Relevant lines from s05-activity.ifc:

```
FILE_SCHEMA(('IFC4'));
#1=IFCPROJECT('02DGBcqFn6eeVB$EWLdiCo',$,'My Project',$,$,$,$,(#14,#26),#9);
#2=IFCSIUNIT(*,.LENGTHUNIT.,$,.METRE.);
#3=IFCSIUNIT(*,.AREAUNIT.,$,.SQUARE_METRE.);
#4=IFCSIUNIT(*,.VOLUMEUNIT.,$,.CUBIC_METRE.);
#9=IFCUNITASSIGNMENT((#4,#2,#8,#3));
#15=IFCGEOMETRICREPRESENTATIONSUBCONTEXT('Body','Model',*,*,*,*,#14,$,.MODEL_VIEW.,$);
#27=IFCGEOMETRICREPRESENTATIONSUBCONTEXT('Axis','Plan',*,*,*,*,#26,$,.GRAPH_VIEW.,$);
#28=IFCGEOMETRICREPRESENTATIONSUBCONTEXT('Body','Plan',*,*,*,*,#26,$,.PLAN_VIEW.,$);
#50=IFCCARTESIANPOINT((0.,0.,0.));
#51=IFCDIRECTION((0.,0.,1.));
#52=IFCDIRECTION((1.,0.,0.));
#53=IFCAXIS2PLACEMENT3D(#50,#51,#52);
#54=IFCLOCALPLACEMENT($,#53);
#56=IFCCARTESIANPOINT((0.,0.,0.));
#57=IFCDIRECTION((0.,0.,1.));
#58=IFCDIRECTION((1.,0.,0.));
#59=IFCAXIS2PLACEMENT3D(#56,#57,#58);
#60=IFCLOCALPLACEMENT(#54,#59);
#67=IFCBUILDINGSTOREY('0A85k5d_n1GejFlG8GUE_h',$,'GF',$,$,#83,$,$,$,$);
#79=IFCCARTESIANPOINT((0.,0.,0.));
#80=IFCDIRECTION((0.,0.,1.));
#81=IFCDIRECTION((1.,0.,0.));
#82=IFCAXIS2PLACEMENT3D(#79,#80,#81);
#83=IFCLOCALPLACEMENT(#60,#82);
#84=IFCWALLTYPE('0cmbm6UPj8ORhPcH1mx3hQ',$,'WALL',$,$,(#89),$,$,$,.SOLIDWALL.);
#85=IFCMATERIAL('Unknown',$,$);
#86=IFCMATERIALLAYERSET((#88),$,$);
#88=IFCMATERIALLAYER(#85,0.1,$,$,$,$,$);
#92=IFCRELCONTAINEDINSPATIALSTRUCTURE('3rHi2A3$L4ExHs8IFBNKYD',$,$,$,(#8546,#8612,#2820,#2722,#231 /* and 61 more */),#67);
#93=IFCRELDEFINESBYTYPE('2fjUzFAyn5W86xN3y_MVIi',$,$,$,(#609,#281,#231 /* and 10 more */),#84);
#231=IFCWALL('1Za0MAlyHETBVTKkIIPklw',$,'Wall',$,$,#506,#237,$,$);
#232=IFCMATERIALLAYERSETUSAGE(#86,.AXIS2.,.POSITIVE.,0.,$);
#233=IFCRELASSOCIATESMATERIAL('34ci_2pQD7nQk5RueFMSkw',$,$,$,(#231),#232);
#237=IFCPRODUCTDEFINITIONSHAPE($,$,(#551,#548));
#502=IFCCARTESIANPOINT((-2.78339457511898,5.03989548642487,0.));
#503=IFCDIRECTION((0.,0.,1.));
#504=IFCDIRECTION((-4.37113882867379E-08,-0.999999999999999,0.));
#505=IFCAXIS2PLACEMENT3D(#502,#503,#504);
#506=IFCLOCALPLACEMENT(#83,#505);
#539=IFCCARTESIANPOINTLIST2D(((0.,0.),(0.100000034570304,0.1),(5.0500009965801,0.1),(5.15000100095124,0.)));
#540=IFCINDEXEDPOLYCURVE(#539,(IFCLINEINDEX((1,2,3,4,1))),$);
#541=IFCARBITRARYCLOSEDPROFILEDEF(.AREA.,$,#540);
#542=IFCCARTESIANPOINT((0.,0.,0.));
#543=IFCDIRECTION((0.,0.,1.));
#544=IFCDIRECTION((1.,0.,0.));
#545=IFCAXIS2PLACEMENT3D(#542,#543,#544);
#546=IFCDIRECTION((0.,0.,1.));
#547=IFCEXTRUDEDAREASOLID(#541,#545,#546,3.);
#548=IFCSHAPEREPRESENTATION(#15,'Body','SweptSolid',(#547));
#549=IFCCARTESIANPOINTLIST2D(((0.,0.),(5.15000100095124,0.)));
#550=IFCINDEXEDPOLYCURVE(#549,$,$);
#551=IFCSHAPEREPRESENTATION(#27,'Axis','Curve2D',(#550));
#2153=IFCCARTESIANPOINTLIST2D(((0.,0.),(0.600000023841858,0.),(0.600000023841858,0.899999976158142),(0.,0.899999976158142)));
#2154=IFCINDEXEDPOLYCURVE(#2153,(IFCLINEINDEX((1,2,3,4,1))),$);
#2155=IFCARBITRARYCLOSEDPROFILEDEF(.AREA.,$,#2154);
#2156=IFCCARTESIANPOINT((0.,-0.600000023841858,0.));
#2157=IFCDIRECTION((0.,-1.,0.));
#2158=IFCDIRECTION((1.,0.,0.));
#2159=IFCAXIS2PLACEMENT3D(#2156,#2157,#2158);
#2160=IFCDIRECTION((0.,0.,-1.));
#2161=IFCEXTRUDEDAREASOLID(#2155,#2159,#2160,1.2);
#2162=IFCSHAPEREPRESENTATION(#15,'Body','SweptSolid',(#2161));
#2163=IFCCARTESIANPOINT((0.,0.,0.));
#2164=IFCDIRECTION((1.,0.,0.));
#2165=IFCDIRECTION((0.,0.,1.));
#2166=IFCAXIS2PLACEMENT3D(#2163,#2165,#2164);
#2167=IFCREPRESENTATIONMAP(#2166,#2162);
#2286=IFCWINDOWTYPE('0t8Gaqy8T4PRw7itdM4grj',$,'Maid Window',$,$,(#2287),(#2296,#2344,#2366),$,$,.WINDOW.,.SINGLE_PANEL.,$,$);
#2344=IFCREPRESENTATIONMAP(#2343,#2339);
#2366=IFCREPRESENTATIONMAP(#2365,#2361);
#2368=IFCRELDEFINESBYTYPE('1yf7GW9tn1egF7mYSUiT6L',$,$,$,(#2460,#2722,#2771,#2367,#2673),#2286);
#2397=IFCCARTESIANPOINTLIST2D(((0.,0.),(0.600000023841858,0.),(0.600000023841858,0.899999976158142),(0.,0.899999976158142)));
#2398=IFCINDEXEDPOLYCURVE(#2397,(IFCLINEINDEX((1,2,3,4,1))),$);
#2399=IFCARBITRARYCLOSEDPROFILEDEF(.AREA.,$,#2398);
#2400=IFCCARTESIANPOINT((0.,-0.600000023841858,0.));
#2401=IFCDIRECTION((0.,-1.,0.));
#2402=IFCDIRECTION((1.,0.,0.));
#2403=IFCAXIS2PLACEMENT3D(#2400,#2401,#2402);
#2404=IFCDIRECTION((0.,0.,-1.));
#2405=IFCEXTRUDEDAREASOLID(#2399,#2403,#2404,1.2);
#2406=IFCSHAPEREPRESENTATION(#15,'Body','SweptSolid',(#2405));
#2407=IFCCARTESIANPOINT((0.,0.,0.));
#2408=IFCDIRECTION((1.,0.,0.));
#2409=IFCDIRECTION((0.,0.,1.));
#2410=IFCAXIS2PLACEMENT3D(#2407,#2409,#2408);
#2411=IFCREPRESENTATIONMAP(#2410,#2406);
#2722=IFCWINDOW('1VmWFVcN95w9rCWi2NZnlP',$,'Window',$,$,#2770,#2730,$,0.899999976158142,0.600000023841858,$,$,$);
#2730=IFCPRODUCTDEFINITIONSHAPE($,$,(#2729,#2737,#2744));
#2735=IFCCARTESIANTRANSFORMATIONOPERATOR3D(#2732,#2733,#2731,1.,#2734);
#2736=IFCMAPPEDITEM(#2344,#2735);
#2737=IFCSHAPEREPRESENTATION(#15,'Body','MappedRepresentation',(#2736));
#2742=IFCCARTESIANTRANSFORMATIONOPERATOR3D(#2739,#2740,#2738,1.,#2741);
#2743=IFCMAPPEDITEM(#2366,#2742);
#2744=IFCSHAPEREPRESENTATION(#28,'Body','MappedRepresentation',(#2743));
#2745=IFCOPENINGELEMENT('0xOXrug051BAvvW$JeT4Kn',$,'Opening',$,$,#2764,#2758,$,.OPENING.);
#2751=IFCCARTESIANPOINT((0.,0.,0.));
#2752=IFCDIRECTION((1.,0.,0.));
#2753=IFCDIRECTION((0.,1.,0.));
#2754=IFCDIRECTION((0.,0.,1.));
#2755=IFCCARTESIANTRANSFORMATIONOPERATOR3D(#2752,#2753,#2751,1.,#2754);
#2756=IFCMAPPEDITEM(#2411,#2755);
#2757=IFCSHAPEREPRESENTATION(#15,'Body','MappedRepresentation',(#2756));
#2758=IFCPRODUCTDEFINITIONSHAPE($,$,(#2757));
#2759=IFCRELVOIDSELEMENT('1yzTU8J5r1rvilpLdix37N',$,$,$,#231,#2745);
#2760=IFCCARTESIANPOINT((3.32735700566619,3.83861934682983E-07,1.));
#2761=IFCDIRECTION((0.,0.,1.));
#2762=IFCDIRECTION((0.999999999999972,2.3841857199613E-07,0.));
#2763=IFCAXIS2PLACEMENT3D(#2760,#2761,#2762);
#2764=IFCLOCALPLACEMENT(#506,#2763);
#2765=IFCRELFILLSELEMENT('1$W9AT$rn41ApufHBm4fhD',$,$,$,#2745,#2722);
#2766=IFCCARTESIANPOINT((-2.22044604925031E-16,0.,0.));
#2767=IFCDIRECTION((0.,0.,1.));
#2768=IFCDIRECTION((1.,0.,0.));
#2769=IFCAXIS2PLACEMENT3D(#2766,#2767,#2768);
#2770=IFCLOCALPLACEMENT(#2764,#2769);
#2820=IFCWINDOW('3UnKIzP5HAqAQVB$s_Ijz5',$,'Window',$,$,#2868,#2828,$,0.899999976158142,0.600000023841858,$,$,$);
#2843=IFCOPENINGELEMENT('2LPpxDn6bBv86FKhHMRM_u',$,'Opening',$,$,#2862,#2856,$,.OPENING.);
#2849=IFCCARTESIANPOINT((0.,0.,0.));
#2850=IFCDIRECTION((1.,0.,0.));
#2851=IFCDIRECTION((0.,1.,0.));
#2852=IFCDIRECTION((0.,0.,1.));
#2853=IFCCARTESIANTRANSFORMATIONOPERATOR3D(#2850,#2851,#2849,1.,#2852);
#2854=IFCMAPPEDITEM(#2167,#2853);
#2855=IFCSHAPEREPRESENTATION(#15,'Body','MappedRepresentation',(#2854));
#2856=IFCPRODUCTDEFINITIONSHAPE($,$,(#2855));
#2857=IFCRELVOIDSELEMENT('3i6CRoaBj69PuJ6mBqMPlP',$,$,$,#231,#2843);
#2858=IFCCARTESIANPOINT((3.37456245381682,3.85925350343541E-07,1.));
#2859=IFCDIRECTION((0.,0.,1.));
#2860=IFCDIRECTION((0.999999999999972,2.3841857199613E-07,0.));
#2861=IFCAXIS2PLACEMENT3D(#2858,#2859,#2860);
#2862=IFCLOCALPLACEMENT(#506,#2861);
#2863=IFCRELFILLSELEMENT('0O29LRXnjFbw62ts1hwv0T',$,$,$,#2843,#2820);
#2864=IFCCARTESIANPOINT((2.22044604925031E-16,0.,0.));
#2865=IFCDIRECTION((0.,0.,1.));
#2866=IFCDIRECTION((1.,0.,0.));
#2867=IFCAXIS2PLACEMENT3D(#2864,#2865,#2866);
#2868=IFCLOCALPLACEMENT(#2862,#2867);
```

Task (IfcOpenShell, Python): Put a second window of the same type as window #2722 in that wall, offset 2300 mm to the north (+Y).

```python
import ifcopenshell
import ifcopenshell.api.feature
import ifcopenshell.api.geometry
import ifcopenshell.api.root
import ifcopenshell.geom
import ifcopenshell.util.element
import ifcopenshell.util.placement
import ifcopenshell.util.shape

model = ifcopenshell.open("s05-activity.ifc")
settings = ifcopenshell.geom.settings()


def volume(element):
    """Net volume in cubic metres, openings subtracted."""
    shape = ifcopenshell.geom.create_shape(settings, element)
    return ifcopenshell.util.shape.get_volume(shape.geometry)


window = model.by_guid("1VmWFVcN95w9rCWi2NZnlP")
opening = window.FillsVoids[0].RelatingOpeningElement
wall = opening.VoidsElements[0].RelatingBuildingElement
before = volume(wall)
shift = ifcopenshell.util.placement.get_local_placement(wall.ObjectPlacement)[:3, 0] * -2.3

# copy_class copies the void relationship, type, container and properties, but no geometry.
new_opening = ifcopenshell.api.root.copy_class(model, product=opening)
new_opening.Representation = ifcopenshell.util.element.copy_deep(
    model, opening.Representation, exclude=["IfcGeometricRepresentationContext", "IfcRepresentationMap"]
)
new_window = ifcopenshell.api.root.copy_class(model, product=window)
new_window.Representation = ifcopenshell.util.element.copy_deep(
    model, window.Representation, exclude=["IfcGeometricRepresentationContext", "IfcRepresentationMap"]
)
ifcopenshell.api.feature.add_filling(model, opening=new_opening, element=new_window)

for old, new in ((opening, new_opening), (window, new_window)):
    matrix = ifcopenshell.util.placement.get_local_placement(old.ObjectPlacement)
    matrix[:3, 3] += shift
    ifcopenshell.api.geometry.edit_object_placement(model, product=new, matrix=matrix, is_si=False)

after = volume(wall)

print(f"wall volume {before:.3f} -> {after:.3f} m3")

model.write("s05-activity_updated.ifc")
```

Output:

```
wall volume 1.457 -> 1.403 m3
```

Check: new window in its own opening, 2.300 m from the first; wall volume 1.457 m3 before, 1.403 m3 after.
